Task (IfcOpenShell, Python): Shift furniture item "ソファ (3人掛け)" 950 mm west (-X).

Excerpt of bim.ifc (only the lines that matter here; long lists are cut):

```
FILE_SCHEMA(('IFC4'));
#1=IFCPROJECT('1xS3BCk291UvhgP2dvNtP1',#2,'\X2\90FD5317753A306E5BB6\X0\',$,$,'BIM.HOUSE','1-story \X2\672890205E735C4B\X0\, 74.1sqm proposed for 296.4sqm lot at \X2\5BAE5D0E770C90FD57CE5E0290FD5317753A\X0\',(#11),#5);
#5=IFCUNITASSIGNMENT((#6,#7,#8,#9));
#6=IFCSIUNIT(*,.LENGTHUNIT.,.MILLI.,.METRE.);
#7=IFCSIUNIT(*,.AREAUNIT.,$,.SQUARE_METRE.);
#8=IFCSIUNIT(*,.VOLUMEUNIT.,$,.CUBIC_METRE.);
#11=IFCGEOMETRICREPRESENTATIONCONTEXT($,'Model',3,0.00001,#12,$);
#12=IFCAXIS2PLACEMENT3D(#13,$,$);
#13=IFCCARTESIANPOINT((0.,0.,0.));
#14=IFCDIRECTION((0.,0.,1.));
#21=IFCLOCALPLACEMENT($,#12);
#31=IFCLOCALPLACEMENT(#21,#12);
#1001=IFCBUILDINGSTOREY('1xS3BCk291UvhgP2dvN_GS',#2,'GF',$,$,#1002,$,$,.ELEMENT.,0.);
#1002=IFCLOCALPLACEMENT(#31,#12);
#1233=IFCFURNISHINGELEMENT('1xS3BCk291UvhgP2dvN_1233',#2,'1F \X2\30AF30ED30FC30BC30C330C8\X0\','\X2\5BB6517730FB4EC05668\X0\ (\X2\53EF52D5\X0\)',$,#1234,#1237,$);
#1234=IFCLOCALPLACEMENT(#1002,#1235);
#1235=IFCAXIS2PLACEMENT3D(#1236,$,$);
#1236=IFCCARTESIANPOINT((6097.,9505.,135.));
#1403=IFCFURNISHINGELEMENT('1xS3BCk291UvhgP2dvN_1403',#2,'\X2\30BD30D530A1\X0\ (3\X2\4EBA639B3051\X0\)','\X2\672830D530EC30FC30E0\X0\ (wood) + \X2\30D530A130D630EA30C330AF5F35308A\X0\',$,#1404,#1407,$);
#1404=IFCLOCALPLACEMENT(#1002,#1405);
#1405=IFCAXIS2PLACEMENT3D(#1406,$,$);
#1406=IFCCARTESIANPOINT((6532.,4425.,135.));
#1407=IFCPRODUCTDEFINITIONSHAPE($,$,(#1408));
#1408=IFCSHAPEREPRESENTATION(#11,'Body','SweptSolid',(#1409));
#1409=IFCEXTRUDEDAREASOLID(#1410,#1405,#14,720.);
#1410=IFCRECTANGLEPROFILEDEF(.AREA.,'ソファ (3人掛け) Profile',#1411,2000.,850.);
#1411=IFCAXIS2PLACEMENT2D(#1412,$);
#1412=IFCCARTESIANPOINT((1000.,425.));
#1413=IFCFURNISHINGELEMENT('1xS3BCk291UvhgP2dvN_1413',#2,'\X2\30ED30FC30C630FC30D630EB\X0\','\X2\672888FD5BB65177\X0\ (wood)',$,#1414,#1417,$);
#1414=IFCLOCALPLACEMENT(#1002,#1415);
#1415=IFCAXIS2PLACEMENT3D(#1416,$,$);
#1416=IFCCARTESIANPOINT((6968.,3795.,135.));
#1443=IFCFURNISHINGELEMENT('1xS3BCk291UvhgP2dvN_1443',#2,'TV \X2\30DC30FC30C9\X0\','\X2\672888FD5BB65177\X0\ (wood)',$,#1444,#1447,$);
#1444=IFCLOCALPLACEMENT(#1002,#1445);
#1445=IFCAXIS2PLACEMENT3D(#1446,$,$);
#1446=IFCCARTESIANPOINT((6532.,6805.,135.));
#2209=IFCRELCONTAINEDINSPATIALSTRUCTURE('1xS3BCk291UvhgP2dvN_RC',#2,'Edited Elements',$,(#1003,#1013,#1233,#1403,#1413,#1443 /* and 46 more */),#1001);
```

```python
import ifcopenshell
import ifcopenshell.api.geometry
import ifcopenshell.util.placement
import ifcopenshell.util.unit

model = ifcopenshell.open("bim.ifc")
unit_scale = ifcopenshell.util.unit.calculate_unit_scale(model)

item = model.by_id(1403)
matrix = ifcopenshell.util.placement.get_local_placement(item.ObjectPlacement)
matrix[0, 3] -= 0.95 / unit_scale
ifcopenshell.api.geometry.edit_object_placement(model, product=item, matrix=matrix, is_si=False)

print(ifcopenshell.util.placement.get_local_placement(item.ObjectPlacement).round(3) + 0.0)

model.write("bim_edited.ifc")
```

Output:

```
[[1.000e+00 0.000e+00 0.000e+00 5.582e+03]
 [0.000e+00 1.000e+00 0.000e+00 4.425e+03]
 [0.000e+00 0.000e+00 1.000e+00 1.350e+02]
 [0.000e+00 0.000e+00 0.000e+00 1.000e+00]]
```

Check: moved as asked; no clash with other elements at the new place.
